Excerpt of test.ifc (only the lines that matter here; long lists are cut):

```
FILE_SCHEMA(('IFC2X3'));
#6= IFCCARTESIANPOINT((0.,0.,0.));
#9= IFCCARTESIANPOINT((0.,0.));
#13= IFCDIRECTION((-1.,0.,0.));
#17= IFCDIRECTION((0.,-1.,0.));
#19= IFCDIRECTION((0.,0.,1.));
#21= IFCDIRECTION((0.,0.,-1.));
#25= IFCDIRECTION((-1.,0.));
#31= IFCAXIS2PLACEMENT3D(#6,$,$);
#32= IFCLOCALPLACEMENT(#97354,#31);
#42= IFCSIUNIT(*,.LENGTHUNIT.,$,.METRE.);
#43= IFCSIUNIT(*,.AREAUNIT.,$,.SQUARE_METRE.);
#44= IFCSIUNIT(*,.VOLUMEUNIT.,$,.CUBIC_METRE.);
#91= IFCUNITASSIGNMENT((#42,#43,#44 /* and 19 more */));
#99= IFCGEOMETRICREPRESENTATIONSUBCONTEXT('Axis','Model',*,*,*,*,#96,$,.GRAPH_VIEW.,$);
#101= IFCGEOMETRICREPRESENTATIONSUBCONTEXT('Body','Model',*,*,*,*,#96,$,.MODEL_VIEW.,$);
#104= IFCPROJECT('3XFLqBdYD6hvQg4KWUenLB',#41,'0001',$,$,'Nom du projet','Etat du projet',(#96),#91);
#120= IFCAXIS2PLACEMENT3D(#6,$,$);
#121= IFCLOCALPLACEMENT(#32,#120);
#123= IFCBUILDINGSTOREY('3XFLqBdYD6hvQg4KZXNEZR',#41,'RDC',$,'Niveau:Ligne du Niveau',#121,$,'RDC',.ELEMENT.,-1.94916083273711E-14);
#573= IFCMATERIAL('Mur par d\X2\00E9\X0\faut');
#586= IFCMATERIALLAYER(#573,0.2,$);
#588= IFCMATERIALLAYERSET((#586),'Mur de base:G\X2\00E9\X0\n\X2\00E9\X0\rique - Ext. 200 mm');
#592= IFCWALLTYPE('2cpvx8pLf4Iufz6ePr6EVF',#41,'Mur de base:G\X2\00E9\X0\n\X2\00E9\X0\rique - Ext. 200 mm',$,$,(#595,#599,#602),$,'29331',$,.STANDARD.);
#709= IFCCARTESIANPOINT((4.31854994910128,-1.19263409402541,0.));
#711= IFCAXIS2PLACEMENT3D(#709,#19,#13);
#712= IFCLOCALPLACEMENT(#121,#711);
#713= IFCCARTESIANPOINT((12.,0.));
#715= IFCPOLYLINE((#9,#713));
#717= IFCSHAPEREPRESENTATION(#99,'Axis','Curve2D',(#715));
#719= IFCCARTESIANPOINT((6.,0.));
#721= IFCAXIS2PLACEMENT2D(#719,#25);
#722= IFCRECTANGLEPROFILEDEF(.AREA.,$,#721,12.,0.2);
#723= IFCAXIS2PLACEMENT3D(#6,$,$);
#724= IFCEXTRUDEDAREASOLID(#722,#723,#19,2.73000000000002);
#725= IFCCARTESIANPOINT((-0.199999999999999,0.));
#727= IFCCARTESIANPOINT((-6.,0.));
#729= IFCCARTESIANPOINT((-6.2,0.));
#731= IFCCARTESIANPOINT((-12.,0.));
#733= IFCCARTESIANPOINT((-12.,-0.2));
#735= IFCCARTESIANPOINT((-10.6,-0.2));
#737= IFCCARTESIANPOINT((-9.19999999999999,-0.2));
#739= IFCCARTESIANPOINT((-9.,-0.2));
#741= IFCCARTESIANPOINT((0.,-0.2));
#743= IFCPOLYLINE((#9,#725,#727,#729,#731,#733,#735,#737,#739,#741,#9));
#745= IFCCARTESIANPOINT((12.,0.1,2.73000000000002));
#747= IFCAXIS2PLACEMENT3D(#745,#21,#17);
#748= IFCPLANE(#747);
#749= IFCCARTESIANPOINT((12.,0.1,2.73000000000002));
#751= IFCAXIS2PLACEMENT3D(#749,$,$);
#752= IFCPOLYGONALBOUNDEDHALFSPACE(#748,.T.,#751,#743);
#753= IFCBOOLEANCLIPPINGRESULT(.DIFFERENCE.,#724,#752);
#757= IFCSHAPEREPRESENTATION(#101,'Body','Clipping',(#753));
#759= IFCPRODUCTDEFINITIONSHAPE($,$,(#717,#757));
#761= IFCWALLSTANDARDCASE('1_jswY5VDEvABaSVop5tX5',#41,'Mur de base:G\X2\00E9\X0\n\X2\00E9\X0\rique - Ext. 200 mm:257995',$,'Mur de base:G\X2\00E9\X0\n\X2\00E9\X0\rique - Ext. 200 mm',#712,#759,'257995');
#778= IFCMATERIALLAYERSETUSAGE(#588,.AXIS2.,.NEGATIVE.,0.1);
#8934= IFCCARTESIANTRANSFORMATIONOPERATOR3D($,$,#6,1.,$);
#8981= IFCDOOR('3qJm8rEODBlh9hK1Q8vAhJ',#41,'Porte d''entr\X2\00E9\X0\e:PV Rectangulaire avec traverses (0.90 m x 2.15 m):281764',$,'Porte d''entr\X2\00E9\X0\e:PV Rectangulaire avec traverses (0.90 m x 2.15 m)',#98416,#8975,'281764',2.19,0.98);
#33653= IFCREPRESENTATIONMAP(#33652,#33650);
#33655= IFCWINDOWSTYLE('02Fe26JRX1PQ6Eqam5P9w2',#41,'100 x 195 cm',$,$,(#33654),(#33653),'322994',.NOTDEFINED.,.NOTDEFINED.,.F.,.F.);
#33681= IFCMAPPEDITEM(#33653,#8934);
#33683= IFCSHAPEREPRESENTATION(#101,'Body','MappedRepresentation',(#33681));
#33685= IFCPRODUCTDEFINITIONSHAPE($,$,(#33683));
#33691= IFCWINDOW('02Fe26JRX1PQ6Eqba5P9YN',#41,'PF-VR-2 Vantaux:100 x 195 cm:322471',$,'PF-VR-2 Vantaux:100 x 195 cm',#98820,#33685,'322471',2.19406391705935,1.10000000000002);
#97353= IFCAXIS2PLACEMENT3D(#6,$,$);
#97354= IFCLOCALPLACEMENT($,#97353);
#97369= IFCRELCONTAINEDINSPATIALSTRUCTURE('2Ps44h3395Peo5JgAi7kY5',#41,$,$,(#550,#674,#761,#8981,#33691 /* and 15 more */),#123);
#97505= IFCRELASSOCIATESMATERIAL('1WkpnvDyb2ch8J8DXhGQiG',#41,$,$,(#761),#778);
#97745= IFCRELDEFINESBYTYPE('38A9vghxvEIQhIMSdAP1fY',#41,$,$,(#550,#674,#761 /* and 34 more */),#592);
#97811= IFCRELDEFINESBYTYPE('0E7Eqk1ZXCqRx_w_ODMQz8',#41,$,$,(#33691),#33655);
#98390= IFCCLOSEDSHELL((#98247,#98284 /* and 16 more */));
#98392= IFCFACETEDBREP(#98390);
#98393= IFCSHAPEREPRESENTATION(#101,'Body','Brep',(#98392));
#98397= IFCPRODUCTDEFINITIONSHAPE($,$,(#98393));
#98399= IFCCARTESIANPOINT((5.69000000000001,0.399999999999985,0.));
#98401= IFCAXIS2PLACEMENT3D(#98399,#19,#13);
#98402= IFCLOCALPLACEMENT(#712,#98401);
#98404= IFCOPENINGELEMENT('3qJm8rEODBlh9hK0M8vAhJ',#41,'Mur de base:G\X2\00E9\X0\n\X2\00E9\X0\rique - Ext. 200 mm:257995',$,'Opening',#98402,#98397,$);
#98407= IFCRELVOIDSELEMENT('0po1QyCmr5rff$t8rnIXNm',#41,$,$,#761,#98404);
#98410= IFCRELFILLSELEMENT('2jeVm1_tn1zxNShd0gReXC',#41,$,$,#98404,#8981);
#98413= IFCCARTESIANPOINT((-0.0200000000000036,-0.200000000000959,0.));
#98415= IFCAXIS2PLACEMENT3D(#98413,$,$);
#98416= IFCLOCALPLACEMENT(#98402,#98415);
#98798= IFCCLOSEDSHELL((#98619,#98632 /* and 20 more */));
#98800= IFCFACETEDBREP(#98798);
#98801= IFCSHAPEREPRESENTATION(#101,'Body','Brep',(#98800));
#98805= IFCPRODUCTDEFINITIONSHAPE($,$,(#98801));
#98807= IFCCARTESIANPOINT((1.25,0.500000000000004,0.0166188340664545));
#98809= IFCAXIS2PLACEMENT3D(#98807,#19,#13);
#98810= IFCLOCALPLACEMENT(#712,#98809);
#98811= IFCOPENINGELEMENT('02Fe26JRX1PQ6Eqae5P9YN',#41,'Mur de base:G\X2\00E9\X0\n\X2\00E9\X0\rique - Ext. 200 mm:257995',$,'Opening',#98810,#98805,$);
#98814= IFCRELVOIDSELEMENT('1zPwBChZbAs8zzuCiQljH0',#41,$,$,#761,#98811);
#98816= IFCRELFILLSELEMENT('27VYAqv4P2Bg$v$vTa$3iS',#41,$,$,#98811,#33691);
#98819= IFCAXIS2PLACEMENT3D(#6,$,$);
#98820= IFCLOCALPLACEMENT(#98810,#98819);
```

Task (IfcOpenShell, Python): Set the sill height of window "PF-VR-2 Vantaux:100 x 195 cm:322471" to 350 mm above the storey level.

```python
import numpy as np
import ifcopenshell
import ifcopenshell.api.geometry
import ifcopenshell.geom
import ifcopenshell.util.element
import ifcopenshell.util.placement
import ifcopenshell.util.shape
import ifcopenshell.util.unit

model = ifcopenshell.open("test.ifc")
unit_scale = ifcopenshell.util.unit.calculate_unit_scale(model)

window = model.by_guid("02Fe26JRX1PQ6Eqba5P9YN")
opening = window.FillsVoids[0].RelatingOpeningElement
storey = ifcopenshell.util.element.get_container(window, ifc_class="IfcBuildingStorey")
level = ifcopenshell.util.placement.get_local_placement(storey.ObjectPlacement)[2, 3]

# The opening's origin need not be at the sill, so measure its lowest point.
shape = ifcopenshell.geom.create_shape(ifcopenshell.geom.settings(), opening)
bottom = ifcopenshell.util.shape.get_shape_bottom_elevation(shape, shape.geometry) / unit_scale
dz = level + 0.35 - bottom

shift = np.array([0.0, 0.0, dz])
# The window is placed relative to its opening, so it follows when the opening moves.
matrix = ifcopenshell.util.placement.get_local_placement(opening.ObjectPlacement)
matrix[:3, 3] += shift
ifcopenshell.api.geometry.edit_object_placement(
    model, product=opening, matrix=matrix, is_si=False, should_transform_children=True
)

print(f"moved by {dz * unit_scale:+.3f} m")

model.write("test_updated.ifc")
```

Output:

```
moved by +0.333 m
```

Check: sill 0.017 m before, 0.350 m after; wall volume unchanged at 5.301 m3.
